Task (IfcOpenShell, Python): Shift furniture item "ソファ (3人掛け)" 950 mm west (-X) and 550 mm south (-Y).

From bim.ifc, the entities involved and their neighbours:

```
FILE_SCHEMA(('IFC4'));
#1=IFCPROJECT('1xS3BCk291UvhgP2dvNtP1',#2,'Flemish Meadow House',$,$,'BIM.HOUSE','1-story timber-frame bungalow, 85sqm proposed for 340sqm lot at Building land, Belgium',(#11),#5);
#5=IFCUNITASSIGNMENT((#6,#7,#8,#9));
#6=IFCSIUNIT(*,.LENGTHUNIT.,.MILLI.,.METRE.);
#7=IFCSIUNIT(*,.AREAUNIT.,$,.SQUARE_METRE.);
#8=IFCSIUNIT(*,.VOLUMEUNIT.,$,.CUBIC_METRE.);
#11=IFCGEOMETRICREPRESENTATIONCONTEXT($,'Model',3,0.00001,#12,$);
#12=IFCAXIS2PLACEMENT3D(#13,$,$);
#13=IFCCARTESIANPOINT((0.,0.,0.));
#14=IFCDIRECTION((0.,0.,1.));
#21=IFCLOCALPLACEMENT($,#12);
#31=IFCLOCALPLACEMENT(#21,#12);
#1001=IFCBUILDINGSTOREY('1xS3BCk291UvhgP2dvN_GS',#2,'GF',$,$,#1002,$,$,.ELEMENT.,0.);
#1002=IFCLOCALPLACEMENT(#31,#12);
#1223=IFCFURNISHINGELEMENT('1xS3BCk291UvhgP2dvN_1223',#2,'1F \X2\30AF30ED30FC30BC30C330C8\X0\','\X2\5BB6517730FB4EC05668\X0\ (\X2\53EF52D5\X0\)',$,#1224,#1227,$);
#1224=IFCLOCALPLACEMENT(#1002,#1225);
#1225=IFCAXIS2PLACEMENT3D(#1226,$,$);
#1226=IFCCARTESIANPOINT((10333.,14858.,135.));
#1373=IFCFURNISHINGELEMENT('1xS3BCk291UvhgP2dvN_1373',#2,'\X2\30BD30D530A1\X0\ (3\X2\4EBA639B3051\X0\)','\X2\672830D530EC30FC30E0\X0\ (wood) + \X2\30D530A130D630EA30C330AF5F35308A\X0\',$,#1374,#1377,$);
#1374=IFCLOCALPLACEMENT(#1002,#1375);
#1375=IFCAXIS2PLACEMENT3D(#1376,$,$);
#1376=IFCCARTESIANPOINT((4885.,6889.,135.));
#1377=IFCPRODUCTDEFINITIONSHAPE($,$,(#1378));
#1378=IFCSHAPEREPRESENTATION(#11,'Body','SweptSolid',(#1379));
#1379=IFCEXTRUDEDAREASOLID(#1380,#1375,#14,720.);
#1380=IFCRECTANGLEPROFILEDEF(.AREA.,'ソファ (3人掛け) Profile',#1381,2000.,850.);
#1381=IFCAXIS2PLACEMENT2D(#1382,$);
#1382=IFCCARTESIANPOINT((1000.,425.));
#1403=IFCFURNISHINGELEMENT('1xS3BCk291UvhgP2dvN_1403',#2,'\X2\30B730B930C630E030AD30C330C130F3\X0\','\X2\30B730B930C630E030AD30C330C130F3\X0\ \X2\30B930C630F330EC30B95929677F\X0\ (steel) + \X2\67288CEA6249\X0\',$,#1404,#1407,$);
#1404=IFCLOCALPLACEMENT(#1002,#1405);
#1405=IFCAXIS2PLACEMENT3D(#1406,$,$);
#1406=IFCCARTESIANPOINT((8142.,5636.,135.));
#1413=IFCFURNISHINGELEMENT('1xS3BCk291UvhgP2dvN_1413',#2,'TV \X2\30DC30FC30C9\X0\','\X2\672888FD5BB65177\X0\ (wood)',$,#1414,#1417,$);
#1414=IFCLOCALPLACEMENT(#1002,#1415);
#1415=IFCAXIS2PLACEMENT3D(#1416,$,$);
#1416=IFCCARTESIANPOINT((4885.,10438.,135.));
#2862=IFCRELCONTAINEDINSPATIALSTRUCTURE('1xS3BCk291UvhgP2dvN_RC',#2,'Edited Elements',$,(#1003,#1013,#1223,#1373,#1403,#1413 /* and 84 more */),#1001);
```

```python
import ifcopenshell
import ifcopenshell.api.geometry
import ifcopenshell.util.placement

model = ifcopenshell.open("bim.ifc")

item = model.by_guid("1xS3BCk291UvhgP2dvN_1373")
matrix = ifcopenshell.util.placement.get_local_placement(item.ObjectPlacement)
matrix[0, 3] -= 950.0
matrix[1, 3] -= 550.0
ifcopenshell.api.geometry.edit_object_placement(model, product=item, matrix=matrix, is_si=False)

print(ifcopenshell.util.placement.get_local_placement(item.ObjectPlacement).round(3) + 0.0)

model.write("bim_edited.ifc")
```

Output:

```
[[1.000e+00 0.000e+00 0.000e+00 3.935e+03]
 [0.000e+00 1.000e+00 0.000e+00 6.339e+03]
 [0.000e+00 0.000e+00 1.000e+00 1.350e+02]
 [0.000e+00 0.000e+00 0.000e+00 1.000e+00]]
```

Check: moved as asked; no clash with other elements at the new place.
